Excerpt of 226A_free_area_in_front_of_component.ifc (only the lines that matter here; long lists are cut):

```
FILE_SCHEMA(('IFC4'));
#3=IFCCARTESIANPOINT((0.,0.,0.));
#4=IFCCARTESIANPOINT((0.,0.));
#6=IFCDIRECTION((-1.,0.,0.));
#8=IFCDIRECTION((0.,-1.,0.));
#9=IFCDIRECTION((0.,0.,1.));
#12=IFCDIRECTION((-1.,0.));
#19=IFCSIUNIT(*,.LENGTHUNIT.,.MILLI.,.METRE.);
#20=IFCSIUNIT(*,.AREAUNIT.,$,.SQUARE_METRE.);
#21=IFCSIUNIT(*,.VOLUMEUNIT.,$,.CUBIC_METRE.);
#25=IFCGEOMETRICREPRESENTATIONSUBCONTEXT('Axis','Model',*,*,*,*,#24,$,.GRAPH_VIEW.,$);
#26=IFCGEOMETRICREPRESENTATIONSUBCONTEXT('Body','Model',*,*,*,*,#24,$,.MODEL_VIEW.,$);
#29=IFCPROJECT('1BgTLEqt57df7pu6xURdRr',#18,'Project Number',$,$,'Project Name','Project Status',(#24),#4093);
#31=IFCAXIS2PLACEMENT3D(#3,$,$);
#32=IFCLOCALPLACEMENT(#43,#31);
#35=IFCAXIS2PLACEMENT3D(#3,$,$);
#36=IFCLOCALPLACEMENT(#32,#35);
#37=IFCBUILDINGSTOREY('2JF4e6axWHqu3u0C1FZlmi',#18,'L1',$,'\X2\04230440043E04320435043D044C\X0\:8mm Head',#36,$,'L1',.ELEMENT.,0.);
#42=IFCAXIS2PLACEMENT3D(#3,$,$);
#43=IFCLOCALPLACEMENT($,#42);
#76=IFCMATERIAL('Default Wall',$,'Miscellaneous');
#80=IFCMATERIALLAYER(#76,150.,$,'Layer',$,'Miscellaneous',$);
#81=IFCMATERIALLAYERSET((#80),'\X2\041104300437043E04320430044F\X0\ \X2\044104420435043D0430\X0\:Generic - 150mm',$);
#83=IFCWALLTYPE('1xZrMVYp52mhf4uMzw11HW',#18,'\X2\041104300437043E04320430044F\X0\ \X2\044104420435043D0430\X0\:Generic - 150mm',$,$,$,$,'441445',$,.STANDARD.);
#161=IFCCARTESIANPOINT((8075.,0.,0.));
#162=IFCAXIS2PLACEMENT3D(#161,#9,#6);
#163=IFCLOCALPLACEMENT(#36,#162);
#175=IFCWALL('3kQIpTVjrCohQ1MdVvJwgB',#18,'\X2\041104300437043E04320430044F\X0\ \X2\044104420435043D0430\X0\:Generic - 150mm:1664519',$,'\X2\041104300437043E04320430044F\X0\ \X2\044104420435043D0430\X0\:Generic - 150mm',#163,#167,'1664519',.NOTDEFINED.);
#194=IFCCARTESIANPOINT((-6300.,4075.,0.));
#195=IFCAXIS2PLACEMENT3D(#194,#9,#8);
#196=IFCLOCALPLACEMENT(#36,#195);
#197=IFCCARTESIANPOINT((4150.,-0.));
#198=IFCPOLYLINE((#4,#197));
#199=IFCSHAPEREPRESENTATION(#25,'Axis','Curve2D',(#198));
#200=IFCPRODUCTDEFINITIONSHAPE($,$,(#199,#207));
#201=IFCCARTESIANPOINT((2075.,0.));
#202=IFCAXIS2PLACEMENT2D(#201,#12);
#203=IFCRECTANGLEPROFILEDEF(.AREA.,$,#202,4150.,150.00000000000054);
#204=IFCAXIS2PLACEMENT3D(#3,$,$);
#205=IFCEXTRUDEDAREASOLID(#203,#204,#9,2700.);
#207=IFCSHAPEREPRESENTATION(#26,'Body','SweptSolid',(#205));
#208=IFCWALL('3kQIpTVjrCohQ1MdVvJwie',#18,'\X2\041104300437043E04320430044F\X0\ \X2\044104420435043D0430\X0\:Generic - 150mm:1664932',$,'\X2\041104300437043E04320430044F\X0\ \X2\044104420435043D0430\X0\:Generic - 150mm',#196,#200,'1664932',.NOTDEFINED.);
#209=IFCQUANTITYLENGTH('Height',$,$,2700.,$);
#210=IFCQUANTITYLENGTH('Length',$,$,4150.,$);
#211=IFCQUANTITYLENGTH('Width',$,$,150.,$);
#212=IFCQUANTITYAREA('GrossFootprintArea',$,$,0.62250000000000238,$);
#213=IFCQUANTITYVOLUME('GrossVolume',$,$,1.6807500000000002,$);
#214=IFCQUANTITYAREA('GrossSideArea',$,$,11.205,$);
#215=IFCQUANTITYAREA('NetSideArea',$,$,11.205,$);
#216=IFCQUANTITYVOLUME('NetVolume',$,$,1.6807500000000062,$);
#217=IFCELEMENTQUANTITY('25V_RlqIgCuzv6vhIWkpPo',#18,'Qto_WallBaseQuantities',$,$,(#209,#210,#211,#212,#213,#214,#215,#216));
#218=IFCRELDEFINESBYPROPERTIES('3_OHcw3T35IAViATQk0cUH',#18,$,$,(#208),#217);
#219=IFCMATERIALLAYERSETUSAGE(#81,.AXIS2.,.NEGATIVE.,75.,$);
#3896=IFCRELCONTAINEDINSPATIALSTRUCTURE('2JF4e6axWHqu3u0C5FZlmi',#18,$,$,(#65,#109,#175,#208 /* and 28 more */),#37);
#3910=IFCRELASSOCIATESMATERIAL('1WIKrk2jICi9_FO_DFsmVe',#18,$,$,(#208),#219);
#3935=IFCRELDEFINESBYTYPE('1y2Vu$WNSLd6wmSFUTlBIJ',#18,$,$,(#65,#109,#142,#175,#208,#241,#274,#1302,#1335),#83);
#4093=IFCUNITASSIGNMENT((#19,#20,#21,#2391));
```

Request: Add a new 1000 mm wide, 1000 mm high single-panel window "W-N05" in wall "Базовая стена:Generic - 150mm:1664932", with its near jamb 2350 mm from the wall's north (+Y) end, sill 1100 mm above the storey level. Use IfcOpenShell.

```python
import numpy as np
import ifcopenshell
import ifcopenshell.api.feature
import ifcopenshell.api.geometry
import ifcopenshell.api.pset
import ifcopenshell.api.root
import ifcopenshell.api.spatial
import ifcopenshell.geom
import ifcopenshell.util.element
import ifcopenshell.util.placement
import ifcopenshell.util.representation
import ifcopenshell.util.shape
import ifcopenshell.util.unit

model = ifcopenshell.open("226A_free_area_in_front_of_component.ifc")
unit_scale = ifcopenshell.util.unit.calculate_unit_scale(model)
area_scale = ifcopenshell.util.unit.calculate_unit_scale(model, "AREAUNIT")
volume_scale = ifcopenshell.util.unit.calculate_unit_scale(model, "VOLUMEUNIT")
settings = ifcopenshell.geom.settings()


def volume(element):
    """Net volume in cubic metres, openings subtracted."""
    shape = ifcopenshell.geom.create_shape(settings, element)
    return ifcopenshell.util.shape.get_volume(shape.geometry)


wall = model.by_id(208)
storey = ifcopenshell.util.element.get_container(wall, ifc_class="IfcBuildingStorey")
context = ifcopenshell.util.representation.get_context(model, "Model", "Body", "MODEL_VIEW")
before = volume(wall)

width, height, from_end, sill = 1, 1, 2.35, 1.1  # metres

# The wall runs along its own X axis, and the end named is its -X end.
wall_shape = ifcopenshell.geom.create_shape(settings, wall)
x, y, z = ifcopenshell.util.shape.get_vertices(wall_shape.geometry).T
start = x.min() + from_end
face, thickness = float(y.min()), float(y.max() - y.min())
wall_matrix = ifcopenshell.util.placement.get_local_placement(wall.ObjectPlacement)
level = ifcopenshell.util.placement.get_local_placement(storey.ObjectPlacement)[2, 3]


def in_wall(x, y):
    """Placement at x, y metres in the wall's axes, at sill height."""
    matrix = wall_matrix.copy()
    matrix[:, 3] = wall_matrix @ np.array([x / unit_scale, y / unit_scale, 0.0, 1.0])
    matrix[2, 3] = level + sill / unit_scale
    return matrix


# Opening: a box that overshoots both wall faces by 50 mm.
opening = ifcopenshell.api.root.create_entity(model, ifc_class="IfcOpeningElement", predefined_type="OPENING")
box = ifcopenshell.api.geometry.add_wall_representation(
    model, context=context, length=width, height=height, thickness=thickness + 0.1
)
ifcopenshell.api.geometry.assign_representation(model, product=opening, representation=box)
ifcopenshell.api.geometry.edit_object_placement(model, product=opening, matrix=in_wall(start, face - 0.05), is_si=False)
ifcopenshell.api.feature.add_feature(model, feature=opening, element=wall)

window = ifcopenshell.api.root.create_entity(model, ifc_class="IfcWindow", name="W-N05", predefined_type="WINDOW")
window.OverallWidth, window.OverallHeight = width / unit_scale, height / unit_scale
window.PartitioningType = "SINGLE_PANEL"
body = ifcopenshell.api.geometry.add_window_representation(
    model,
    context=context,
    overall_width=window.OverallWidth,
    overall_height=window.OverallHeight,
    partition_type="SINGLE_PANEL",
)
ifcopenshell.api.geometry.assign_representation(model, product=window, representation=body)
ifcopenshell.api.spatial.assign_container(model, products=[window], relating_structure=storey)
ifcopenshell.api.feature.add_filling(model, opening=opening, element=window)

# Centre the window in the wall's thickness.
ifcopenshell.api.geometry.edit_object_placement(model, product=window, matrix=in_wall(start, face), is_si=False)
window_shape = ifcopenshell.geom.create_shape(settings, window)
depth = ifcopenshell.util.shape.get_vertices(window_shape.geometry)[:, 1]
offset = face + thickness / 2 - (depth.min() + depth.max()) / 2
ifcopenshell.api.geometry.edit_object_placement(model, product=window, matrix=in_wall(start, offset), is_si=False)

after = volume(wall)

# Update the wall's stored quantities.
qto = model.by_id(ifcopenshell.util.element.get_pset(wall, "Qto_WallBaseQuantities", should_inherit=False)["id"])
ifcopenshell.api.pset.edit_qto(model, qto=qto, properties={
    "NetSideArea": after / thickness / area_scale,
    "NetVolume": after / volume_scale,
})

print(f"wall volume {before:.3f} -> {after:.3f} m3")

model.write("226A_free_area_in_front_of_component_updated.ifc")
```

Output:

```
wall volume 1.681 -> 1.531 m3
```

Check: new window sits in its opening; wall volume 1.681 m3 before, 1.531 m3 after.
